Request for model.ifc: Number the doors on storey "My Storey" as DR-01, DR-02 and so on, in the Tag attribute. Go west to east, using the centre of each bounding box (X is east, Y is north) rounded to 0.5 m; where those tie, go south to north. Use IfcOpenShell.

First a look at what the model holds.

```python
import ifcopenshell
import ifcopenshell.util.element
import ifcopenshell.util.placement

model = ifcopenshell.open("model.ifc")
print(model.schema)
storey = next(s for s in model.by_type("IfcBuildingStorey") if s.Name == "My Storey")
doors = [e for e in ifcopenshell.util.element.get_decomposition(storey) if e.is_a("IfcDoor")]
for e in sorted(doors, key=lambda e: e.id()):
    origin = ifcopenshell.util.placement.get_local_placement(e.ObjectPlacement)[:3, 3]
    print(e.id(), e.Tag, e.Name, origin.round(2) + 0.0, sep=" | ")
```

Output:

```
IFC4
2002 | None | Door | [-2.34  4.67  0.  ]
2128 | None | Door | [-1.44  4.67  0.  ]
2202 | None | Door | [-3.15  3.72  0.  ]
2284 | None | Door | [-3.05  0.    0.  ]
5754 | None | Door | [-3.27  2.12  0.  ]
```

```python
import ifcopenshell
import ifcopenshell.geom
import ifcopenshell.util.element
import ifcopenshell.util.shape

model = ifcopenshell.open("model.ifc")
settings = ifcopenshell.geom.settings()
settings.set("use-world-coords", True)


def centre(element):
    shape = ifcopenshell.geom.create_shape(settings, element)
    return ifcopenshell.util.shape.get_bbox_centroid(shape.geometry)


storey = next(s for s in model.by_type("IfcBuildingStorey") if s.Name == "My Storey")
doors = [e for e in ifcopenshell.util.element.get_decomposition(storey) if e.is_a("IfcDoor")]

# Insertion points can sit at a corner or the storey origin, so sort by the geometry (in metres).
centres = {e: centre(e) for e in doors}
doors.sort(key=lambda e: (round(centres[e][0] / 0.5), centres[e][1]))

for i, e in enumerate(doors, start=1):
    number = f"DR-{i:02d}"
    e.Tag = number
    print(e.id(), number)

model.write("model_v2.ifc")
```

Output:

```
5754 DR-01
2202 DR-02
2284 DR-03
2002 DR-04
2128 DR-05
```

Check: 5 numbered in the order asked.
